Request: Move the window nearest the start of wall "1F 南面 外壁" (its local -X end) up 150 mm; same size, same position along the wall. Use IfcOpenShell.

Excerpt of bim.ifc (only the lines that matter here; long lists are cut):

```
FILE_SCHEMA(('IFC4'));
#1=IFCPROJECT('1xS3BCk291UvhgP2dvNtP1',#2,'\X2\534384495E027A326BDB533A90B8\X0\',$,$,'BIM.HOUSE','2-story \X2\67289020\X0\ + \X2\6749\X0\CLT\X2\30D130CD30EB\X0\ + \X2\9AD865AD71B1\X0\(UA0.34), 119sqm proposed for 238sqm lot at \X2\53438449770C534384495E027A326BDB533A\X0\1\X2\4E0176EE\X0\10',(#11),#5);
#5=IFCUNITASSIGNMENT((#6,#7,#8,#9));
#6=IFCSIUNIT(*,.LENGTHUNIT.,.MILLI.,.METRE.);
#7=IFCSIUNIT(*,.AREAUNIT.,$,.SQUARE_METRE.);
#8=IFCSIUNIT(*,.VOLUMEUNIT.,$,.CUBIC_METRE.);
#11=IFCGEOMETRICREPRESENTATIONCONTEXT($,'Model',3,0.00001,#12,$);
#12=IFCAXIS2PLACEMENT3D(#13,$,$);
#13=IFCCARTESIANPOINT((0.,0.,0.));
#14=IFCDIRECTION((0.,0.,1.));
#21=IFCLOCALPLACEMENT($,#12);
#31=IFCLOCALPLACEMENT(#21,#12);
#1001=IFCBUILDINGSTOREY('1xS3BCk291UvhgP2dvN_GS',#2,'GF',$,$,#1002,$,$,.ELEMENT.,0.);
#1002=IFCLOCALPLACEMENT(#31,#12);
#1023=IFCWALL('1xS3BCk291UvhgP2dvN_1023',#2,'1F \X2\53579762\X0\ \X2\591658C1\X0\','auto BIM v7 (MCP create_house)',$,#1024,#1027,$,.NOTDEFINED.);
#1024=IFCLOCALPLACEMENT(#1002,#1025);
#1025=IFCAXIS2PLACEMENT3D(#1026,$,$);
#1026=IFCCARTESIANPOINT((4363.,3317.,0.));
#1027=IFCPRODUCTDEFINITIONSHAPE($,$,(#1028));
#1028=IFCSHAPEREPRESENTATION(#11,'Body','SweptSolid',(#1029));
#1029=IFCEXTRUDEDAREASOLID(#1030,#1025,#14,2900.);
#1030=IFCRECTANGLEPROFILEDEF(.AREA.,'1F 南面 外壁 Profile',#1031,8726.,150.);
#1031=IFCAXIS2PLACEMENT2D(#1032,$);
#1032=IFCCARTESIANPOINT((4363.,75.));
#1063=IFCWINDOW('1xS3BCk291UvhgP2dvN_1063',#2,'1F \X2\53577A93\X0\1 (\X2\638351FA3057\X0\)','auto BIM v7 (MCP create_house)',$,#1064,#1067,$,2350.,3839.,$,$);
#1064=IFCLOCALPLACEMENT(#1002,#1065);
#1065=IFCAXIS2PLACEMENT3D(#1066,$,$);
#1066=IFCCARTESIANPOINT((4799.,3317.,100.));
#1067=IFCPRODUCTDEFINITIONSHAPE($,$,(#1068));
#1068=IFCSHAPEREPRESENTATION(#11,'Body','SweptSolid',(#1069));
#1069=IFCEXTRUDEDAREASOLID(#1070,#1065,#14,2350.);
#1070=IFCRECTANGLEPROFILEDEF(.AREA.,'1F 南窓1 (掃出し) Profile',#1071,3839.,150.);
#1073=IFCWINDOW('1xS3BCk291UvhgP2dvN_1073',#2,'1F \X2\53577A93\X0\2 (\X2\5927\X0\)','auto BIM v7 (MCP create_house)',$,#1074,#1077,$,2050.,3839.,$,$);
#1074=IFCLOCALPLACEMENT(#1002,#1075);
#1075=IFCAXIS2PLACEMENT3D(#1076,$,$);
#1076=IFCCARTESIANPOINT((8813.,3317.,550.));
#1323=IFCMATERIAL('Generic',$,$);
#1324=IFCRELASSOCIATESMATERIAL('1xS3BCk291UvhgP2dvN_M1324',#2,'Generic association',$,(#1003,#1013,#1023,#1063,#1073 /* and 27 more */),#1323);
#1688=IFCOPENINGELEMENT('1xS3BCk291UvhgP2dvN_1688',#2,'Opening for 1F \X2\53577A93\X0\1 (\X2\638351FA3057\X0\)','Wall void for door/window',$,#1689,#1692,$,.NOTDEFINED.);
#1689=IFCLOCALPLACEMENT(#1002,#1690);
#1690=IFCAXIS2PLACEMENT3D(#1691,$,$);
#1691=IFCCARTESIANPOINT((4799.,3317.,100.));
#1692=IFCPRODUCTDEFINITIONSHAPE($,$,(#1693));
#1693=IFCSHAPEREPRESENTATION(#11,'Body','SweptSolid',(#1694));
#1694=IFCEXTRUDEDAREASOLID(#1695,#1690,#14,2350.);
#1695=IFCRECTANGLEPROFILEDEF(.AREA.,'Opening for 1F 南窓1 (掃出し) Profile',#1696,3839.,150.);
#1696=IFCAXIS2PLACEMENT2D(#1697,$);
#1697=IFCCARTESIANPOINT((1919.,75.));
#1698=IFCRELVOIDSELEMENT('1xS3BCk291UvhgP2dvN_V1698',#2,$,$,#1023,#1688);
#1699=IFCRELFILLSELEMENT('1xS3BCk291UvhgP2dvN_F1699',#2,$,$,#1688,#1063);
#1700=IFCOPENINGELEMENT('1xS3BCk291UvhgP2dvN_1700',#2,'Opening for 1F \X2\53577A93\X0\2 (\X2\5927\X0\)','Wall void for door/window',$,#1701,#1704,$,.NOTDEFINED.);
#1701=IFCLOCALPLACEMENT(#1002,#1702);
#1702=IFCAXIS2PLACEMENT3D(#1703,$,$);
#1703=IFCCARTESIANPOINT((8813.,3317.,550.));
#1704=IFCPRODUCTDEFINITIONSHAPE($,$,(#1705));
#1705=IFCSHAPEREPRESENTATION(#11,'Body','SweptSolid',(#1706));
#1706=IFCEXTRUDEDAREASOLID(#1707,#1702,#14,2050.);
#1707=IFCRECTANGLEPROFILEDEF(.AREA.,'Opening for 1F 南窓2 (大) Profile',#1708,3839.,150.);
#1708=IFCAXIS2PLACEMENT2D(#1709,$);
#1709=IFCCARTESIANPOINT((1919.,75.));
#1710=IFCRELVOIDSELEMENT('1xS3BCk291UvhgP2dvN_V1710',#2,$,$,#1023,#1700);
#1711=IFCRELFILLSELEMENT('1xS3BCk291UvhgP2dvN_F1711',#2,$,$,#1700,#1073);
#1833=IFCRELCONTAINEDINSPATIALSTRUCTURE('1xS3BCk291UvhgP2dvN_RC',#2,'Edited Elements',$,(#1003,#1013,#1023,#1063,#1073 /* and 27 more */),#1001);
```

```python
import numpy as np
import ifcopenshell
import ifcopenshell.api.geometry
import ifcopenshell.util.placement
import ifcopenshell.util.unit

model = ifcopenshell.open("bim.ifc")
unit_scale = ifcopenshell.util.unit.calculate_unit_scale(model)

window = model.by_id(1063)
opening = window.FillsVoids[0].RelatingOpeningElement
dz = 0.15 / unit_scale

shift = np.array([0.0, 0.0, dz])
# The window is not placed relative to its opening, so move both.
for product in (opening, window):
    matrix = ifcopenshell.util.placement.get_local_placement(product.ObjectPlacement)
    matrix[:3, 3] += shift
    ifcopenshell.api.geometry.edit_object_placement(model, product=product, matrix=matrix, is_si=False)

print(f"moved by {dz * unit_scale:+.3f} m")

model.write("bim_v2.ifc")
```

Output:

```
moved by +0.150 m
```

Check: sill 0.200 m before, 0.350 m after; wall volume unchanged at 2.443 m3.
